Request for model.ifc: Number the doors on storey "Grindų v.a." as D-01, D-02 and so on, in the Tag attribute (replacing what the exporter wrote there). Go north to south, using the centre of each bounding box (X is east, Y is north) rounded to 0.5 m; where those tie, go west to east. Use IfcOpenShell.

First a look at what the model holds.

```python
import ifcopenshell
import ifcopenshell.util.element
import ifcopenshell.util.placement

model = ifcopenshell.open("model.ifc")
print(model.schema)
storey = next(s for s in model.by_type("IfcBuildingStorey") if s.Name == "Grindų v.a.")
doors = [e for e in ifcopenshell.util.element.get_decomposition(storey) if e.is_a("IfcDoor")]
for e in sorted(doors, key=lambda e: e.id()):
    origin = ifcopenshell.util.placement.get_local_placement(e.ObjectPlacement)[:3, 3]
    print(e.id(), e.Tag, e.Name, origin.round(2) + 0.0, sep=" | ")
```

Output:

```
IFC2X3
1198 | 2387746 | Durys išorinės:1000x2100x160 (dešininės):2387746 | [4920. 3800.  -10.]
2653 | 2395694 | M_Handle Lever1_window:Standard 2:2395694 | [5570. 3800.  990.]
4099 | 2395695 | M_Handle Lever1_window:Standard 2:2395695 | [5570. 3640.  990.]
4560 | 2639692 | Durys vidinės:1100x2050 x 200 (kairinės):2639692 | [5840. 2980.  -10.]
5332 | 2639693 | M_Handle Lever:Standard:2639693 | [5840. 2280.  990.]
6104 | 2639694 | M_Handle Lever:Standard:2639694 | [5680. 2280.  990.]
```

```python
import ifcopenshell
import ifcopenshell.geom
import ifcopenshell.util.element
import ifcopenshell.util.shape

model = ifcopenshell.open("model.ifc")
settings = ifcopenshell.geom.settings()
settings.set("use-world-coords", True)


def centre(element):
    shape = ifcopenshell.geom.create_shape(settings, element)
    return ifcopenshell.util.shape.get_bbox_centroid(shape.geometry)


storey = next(s for s in model.by_type("IfcBuildingStorey") if s.Name == "Grindų v.a.")
doors = [e for e in ifcopenshell.util.element.get_decomposition(storey) if e.is_a("IfcDoor")]

# Insertion points can sit at a corner or the storey origin, so sort by the geometry (in metres).
centres = {e: centre(e) for e in doors}
doors.sort(key=lambda e: (-round(centres[e][1] / 0.5), centres[e][0]))

for i, e in enumerate(doors, start=1):
    number = f"D-{i:02d}"
    e.Tag = number
    print(e.id(), number)

model.write("model_edited.ifc")
```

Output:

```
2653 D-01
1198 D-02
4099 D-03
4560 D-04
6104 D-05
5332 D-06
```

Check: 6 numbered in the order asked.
